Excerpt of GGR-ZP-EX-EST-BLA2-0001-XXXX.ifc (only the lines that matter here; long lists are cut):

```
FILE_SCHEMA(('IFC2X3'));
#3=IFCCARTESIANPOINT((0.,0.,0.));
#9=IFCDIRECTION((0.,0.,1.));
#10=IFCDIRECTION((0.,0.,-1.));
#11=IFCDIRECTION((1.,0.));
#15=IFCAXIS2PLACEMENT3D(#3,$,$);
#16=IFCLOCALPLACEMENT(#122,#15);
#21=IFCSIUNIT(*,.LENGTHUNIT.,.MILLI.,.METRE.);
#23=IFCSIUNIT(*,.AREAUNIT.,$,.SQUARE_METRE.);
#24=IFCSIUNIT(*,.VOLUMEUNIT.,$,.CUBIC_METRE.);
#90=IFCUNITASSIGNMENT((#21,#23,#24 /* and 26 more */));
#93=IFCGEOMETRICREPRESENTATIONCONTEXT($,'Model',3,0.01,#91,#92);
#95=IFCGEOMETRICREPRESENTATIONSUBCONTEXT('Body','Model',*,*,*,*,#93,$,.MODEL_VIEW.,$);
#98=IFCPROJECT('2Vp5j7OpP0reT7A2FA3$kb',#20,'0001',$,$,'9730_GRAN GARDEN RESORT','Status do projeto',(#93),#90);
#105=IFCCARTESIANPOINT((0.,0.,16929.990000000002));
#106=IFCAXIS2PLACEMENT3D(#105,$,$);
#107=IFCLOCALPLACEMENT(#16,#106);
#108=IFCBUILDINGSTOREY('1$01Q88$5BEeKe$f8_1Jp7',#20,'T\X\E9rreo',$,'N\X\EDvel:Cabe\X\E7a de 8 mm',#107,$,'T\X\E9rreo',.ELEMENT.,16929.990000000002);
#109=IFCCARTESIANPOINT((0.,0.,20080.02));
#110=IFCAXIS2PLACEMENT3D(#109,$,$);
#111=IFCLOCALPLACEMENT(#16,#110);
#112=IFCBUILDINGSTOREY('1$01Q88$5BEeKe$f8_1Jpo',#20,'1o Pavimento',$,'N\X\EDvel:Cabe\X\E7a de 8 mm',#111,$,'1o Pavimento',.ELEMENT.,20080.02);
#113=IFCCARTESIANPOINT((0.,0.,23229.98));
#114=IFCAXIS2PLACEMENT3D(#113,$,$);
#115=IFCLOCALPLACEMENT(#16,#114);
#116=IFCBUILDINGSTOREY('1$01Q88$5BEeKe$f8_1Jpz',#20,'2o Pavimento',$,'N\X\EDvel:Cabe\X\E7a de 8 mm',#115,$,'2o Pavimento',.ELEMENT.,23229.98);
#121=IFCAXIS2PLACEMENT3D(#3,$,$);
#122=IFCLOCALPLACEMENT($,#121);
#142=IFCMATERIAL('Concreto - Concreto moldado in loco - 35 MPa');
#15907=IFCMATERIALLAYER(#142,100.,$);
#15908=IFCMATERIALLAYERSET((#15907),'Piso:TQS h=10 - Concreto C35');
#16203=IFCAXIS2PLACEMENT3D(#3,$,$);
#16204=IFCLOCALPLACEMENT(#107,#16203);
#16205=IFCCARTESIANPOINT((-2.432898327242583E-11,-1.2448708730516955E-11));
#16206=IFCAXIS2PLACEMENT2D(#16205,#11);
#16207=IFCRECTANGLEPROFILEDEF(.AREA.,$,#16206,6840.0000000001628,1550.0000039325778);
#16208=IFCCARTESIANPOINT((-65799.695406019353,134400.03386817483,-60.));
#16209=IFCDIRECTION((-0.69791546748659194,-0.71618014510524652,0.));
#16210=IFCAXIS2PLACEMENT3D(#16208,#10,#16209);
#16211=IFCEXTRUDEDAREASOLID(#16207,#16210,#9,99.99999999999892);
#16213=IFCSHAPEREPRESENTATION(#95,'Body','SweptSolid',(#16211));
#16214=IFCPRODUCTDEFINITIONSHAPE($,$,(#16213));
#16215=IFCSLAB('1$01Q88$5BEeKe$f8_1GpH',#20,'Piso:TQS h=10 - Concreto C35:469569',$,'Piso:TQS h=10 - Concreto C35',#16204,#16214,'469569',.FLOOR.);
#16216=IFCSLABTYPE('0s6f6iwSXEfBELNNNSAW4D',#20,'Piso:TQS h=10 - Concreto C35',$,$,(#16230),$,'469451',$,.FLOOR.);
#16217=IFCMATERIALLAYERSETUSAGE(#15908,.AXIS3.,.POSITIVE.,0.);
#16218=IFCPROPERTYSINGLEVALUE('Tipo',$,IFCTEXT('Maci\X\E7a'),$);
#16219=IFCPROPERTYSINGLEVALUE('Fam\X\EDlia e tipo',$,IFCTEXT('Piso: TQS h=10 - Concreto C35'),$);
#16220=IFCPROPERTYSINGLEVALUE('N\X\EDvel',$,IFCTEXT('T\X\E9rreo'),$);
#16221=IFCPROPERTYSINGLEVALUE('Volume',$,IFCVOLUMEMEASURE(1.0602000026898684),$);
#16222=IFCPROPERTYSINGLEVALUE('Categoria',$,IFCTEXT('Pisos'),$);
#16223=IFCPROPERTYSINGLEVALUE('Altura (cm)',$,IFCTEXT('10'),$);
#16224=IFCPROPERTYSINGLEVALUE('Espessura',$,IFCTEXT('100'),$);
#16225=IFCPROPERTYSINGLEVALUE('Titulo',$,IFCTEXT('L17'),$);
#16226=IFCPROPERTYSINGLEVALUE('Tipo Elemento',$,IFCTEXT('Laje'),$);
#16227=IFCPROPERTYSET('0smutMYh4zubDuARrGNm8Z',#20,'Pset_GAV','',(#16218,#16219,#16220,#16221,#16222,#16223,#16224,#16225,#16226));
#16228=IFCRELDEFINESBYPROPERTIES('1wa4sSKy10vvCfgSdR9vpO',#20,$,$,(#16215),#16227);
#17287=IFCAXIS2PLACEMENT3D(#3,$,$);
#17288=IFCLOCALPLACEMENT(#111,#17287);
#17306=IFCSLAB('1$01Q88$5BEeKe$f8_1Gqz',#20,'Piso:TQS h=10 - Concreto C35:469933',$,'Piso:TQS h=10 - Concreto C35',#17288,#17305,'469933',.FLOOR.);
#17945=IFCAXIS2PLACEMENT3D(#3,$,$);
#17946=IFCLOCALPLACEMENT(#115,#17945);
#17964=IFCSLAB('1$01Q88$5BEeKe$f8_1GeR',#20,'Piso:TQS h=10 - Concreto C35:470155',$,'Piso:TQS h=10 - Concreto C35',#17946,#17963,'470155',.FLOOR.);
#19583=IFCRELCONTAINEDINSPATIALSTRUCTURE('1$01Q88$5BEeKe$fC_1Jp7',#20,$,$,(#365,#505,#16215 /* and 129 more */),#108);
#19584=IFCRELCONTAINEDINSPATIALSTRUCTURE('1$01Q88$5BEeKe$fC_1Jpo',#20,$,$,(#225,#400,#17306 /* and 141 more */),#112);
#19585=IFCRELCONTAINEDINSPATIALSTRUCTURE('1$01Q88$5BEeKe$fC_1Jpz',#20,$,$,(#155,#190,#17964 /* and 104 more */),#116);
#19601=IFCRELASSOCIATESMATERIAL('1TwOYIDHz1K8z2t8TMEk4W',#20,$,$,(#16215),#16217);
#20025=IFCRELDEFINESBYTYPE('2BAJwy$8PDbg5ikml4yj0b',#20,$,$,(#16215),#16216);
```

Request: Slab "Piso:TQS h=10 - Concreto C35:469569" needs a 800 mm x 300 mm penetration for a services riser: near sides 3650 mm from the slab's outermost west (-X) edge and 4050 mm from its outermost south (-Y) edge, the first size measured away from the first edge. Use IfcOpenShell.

```python
import numpy as np
import ifcopenshell
import ifcopenshell.api.feature
import ifcopenshell.api.geometry
import ifcopenshell.api.pset
import ifcopenshell.api.root
import ifcopenshell.geom
import ifcopenshell.util.element
import ifcopenshell.util.placement
import ifcopenshell.util.representation
import ifcopenshell.util.shape
import ifcopenshell.util.unit

model = ifcopenshell.open("GGR-ZP-EX-EST-BLA2-0001-XXXX.ifc")
unit_scale = ifcopenshell.util.unit.calculate_unit_scale(model)
volume_scale = ifcopenshell.util.unit.calculate_unit_scale(model, "VOLUMEUNIT")
settings = ifcopenshell.geom.settings()


def volume(element):
    """Net volume in cubic metres, openings subtracted."""
    shape = ifcopenshell.geom.create_shape(settings, element)
    return ifcopenshell.util.shape.get_volume(shape.geometry)


slab = model.by_id(16215)
before = volume(slab)

# Extent in the slab's own axes, in metres. The edges named are its -X and -Y sides.
slab_shape = ifcopenshell.geom.create_shape(settings, slab)
vertices = ifcopenshell.util.shape.get_vertices(slab_shape.geometry)
x_min, y_min, bottom = vertices.min(axis=0)
top = vertices[:, 2].max()

opening = ifcopenshell.api.root.create_entity(model, ifc_class="IfcOpeningElement", name="Services riser opening")
context = ifcopenshell.util.representation.get_context(model, "Model", "Body", "MODEL_VIEW")
width, depth = 0.8, 0.3
outline = [(0.0, 0.0), (width, 0.0), (width, depth), (0.0, depth), (0.0, 0.0)]
# Overshoot both faces by 50 mm so the cut is clean.
shape = ifcopenshell.api.geometry.add_slab_representation(
    model, context=context, depth=top - bottom + 0.1, polyline=outline
)
ifcopenshell.api.geometry.assign_representation(model, product=opening, representation=shape)

matrix = ifcopenshell.util.placement.get_local_placement(slab.ObjectPlacement)
matrix[:, 3] = matrix @ np.append(np.array([x_min + 3.65, y_min + 4.05, bottom - 0.05]) / unit_scale, 1.0)
ifcopenshell.api.geometry.edit_object_placement(model, product=opening, matrix=matrix, is_si=False)
ifcopenshell.api.feature.add_feature(model, feature=opening, element=slab)

after = volume(slab)

# Update the slab's stored quantities.
pset = model.by_id(ifcopenshell.util.element.get_pset(slab, "Pset_GAV", should_inherit=False)["id"])
ifcopenshell.api.pset.edit_pset(model, pset=pset, properties={
    "Volume": model.create_entity("IfcVolumeMeasure", after / volume_scale),
})

print(f"slab volume {before:.3f} -> {after:.3f} m3")

model.write("GGR-ZP-EX-EST-BLA2-0001-XXXX_edited.ifc")
```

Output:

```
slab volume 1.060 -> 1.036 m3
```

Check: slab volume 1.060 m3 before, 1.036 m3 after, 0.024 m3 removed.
